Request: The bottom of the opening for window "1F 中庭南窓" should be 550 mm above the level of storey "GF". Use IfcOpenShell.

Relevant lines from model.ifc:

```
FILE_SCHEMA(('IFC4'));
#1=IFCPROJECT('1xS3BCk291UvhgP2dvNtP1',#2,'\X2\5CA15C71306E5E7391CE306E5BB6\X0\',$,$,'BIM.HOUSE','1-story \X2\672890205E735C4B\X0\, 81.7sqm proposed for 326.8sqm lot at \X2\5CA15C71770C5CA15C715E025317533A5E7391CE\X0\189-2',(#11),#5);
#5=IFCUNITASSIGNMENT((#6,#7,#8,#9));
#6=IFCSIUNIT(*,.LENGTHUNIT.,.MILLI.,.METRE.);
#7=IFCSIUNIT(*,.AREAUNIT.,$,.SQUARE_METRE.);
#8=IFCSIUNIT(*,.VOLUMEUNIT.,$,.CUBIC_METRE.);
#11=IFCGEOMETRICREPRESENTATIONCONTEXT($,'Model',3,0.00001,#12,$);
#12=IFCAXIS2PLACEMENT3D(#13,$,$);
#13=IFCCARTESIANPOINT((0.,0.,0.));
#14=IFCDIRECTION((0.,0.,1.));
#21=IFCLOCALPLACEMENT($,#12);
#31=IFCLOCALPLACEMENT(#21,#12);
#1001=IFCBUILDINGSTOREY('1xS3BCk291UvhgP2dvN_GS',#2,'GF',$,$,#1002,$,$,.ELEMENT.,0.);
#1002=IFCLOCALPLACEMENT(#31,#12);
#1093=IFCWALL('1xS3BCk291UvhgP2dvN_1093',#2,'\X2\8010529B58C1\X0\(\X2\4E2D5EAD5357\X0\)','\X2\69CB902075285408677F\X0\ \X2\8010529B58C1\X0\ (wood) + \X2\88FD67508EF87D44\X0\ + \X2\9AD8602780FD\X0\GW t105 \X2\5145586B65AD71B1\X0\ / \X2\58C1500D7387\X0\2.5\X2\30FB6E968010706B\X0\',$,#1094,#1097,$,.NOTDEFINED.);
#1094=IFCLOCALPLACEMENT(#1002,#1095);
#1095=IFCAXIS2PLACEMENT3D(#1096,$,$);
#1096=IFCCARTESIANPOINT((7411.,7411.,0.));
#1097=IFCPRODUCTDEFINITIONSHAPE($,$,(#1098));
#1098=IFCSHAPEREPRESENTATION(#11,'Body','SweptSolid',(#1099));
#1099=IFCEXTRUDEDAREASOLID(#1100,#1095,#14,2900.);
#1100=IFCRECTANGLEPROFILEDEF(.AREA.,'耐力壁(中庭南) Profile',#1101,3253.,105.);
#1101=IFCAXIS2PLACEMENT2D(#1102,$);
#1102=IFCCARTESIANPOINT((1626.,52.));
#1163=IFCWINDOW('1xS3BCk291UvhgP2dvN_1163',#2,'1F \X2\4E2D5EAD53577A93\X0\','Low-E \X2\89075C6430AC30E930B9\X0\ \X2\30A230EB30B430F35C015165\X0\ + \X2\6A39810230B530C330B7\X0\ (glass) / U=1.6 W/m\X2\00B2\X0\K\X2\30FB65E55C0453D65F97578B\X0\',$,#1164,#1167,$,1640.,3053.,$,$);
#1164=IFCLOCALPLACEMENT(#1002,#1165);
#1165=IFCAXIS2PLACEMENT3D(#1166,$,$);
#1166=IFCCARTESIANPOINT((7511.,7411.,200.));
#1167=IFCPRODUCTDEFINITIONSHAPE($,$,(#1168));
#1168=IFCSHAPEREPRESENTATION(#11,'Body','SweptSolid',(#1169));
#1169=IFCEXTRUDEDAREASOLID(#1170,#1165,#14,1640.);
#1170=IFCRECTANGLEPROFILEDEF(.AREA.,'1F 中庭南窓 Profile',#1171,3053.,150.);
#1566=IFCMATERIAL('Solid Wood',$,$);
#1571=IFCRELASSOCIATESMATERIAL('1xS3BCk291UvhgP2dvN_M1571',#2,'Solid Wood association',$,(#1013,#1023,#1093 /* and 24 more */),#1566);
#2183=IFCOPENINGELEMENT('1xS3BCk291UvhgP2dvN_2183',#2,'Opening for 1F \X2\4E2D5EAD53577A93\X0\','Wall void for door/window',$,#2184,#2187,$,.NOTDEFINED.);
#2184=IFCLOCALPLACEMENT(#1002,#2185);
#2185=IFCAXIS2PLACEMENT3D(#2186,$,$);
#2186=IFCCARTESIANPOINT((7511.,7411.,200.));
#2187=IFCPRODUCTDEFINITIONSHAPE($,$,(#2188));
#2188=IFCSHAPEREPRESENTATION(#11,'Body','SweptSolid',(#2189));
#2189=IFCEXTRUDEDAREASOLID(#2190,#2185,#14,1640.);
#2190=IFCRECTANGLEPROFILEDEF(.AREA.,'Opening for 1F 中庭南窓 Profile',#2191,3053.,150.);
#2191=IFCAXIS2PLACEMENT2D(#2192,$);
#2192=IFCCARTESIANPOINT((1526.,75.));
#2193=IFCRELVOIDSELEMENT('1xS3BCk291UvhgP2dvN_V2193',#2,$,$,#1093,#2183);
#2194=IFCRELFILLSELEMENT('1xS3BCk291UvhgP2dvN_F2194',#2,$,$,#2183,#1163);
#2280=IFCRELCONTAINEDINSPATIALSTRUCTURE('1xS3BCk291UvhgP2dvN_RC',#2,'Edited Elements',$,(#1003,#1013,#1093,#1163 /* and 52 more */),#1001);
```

```python
import numpy as np
import ifcopenshell
import ifcopenshell.api.geometry
import ifcopenshell.geom
import ifcopenshell.util.element
import ifcopenshell.util.placement
import ifcopenshell.util.shape
import ifcopenshell.util.unit

model = ifcopenshell.open("model.ifc")
unit_scale = ifcopenshell.util.unit.calculate_unit_scale(model)

window = model.by_id(1163)
opening = window.FillsVoids[0].RelatingOpeningElement
storey = ifcopenshell.util.element.get_container(window, ifc_class="IfcBuildingStorey")
level = ifcopenshell.util.placement.get_local_placement(storey.ObjectPlacement)[2, 3]

# The opening's origin need not be at the sill, so measure its lowest point.
shape = ifcopenshell.geom.create_shape(ifcopenshell.geom.settings(), opening)
bottom = ifcopenshell.util.shape.get_shape_bottom_elevation(shape, shape.geometry) / unit_scale
dz = level + 0.55 / unit_scale - bottom

shift = np.array([0.0, 0.0, dz])
# The window is not placed relative to its opening, so move both.
for product in (opening, window):
    matrix = ifcopenshell.util.placement.get_local_placement(product.ObjectPlacement)
    matrix[:3, 3] += shift
    ifcopenshell.api.geometry.edit_object_placement(model, product=product, matrix=matrix, is_si=False)

print(f"moved by {dz * unit_scale:+.3f} m")

model.write("model_v2.ifc")
```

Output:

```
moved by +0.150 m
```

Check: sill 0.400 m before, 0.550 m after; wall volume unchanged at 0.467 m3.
